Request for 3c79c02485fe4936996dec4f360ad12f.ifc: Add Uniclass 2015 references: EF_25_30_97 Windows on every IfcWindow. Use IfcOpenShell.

First a look at what the model holds.

```python
import ifcopenshell

model = ifcopenshell.open("3c79c02485fe4936996dec4f360ad12f.ifc")
print(model.schema)
print("classifications:", [c.Name for c in model.by_type("IfcClassification")])
for ifc_class in ("IfcDoor", "IfcRoof", "IfcStair", "IfcWall", "IfcWindow"):
    print(ifc_class, len(model.by_type(ifc_class)))
```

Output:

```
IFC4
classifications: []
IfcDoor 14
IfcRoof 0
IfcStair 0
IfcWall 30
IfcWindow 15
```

```python
import ifcopenshell
import ifcopenshell.api.classification

model = ifcopenshell.open("3c79c02485fe4936996dec4f360ad12f.ifc")

system = ifcopenshell.api.classification.add_classification(model, classification="Uniclass 2015")

codes = {
    "IfcWindow": ("EF_25_30_97", "Windows"),
}
for ifc_class, (code, name) in codes.items():
    products = model.by_type(ifc_class)
    ifcopenshell.api.classification.add_reference(
        model, products=products, classification=system, identification=code, name=name
    )
    print(code, len(products))

model.write("3c79c02485fe4936996dec4f360ad12f_v2.ifc")
```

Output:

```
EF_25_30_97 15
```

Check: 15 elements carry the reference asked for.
